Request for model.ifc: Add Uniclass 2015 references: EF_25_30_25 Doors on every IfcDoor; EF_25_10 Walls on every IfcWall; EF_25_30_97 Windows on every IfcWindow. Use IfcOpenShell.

First a look at what the model holds.

```python
import ifcopenshell

model = ifcopenshell.open("model.ifc")
print(model.schema)
print("classifications:", [c.Name for c in model.by_type("IfcClassification")])
for ifc_class in ("IfcDoor", "IfcRoof", "IfcStair", "IfcWall", "IfcWindow"):
    print(ifc_class, len(model.by_type(ifc_class)))
```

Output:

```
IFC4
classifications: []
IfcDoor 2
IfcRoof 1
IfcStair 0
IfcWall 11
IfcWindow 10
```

```python
import ifcopenshell
import ifcopenshell.api.classification

model = ifcopenshell.open("model.ifc")

system = ifcopenshell.api.classification.add_classification(model, classification="Uniclass 2015")

codes = {
    "IfcDoor": ("EF_25_30_25", "Doors"),
    "IfcWall": ("EF_25_10", "Walls"),
    "IfcWindow": ("EF_25_30_97", "Windows"),
}
for ifc_class, (code, name) in codes.items():
    products = model.by_type(ifc_class)
    ifcopenshell.api.classification.add_reference(
        model, products=products, classification=system, identification=code, name=name
    )
    print(code, len(products))

model.write("model_updated.ifc")
```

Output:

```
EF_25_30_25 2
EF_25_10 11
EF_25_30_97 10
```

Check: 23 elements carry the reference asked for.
